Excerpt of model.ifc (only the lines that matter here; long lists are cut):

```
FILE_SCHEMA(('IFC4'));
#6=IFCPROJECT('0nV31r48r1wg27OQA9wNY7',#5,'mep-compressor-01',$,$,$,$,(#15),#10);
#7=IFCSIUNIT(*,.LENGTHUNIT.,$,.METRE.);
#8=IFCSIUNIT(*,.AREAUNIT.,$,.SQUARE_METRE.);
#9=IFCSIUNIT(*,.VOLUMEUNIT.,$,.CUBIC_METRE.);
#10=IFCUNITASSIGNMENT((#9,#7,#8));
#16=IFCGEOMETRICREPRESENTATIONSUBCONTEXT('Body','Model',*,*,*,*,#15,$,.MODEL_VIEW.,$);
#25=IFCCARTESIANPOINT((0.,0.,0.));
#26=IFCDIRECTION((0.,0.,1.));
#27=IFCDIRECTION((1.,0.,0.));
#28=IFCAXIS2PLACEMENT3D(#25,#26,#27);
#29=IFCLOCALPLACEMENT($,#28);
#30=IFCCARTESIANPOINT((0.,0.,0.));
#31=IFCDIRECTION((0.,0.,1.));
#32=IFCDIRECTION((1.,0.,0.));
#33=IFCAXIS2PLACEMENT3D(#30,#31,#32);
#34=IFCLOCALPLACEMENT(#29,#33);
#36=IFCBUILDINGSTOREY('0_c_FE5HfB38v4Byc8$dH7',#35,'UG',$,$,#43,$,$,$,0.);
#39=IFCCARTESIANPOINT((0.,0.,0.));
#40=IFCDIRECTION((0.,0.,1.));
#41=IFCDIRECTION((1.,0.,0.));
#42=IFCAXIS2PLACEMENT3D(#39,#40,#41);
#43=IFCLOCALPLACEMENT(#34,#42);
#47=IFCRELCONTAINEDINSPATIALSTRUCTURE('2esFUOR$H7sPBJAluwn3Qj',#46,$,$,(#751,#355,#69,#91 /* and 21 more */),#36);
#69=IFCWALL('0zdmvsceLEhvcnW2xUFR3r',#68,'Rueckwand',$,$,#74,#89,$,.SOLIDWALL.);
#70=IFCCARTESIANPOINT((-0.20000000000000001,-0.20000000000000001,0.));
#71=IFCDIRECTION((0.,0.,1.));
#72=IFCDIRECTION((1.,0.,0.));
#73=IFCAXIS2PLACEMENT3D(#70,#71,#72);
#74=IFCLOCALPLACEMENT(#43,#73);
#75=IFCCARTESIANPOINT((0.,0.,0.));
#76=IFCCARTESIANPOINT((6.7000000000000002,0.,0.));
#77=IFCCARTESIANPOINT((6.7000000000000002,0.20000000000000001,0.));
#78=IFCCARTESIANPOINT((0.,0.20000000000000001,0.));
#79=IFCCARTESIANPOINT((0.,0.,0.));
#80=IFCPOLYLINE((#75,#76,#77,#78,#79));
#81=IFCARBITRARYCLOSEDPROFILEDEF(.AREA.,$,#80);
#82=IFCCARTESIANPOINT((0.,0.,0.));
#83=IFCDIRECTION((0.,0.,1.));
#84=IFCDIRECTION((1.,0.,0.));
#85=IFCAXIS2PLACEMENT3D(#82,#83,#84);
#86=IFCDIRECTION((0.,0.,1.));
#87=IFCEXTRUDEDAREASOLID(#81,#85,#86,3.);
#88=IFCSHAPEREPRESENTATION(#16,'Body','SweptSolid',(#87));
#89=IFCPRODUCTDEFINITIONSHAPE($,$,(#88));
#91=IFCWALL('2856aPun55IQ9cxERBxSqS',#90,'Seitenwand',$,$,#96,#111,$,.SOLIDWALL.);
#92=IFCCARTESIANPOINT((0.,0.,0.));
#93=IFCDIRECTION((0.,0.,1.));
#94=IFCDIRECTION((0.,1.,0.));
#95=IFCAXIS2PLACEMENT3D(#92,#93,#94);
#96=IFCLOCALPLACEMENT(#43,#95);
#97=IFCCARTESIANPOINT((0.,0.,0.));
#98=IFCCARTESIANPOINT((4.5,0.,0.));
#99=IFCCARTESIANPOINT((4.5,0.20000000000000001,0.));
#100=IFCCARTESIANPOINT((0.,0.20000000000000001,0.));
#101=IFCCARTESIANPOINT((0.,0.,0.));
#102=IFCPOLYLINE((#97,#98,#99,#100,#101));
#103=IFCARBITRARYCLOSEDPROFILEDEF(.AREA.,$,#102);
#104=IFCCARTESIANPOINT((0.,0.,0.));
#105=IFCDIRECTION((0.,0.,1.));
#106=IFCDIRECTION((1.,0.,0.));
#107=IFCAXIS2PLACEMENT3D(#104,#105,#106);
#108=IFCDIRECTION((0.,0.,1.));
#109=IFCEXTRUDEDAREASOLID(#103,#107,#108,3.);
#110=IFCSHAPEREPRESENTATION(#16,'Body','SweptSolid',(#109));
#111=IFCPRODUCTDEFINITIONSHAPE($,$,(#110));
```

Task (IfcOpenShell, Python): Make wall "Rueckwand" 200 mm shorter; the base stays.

```python
import ifcopenshell
import ifcopenshell.geom
import ifcopenshell.util.representation
import ifcopenshell.util.shape

model = ifcopenshell.open("model.ifc")
settings = ifcopenshell.geom.settings()


def volume(element):
    """Net volume in cubic metres, openings subtracted."""
    shape = ifcopenshell.geom.create_shape(settings, element)
    return ifcopenshell.util.shape.get_volume(shape.geometry)


wall = model.by_guid("0zdmvsceLEhvcnW2xUFR3r")
before = volume(wall)

body = ifcopenshell.util.representation.get_representation(wall, "Model", "Body")
solid = body.Items[0]
old_height = solid.Depth
solid.Depth -= 0.2
after = volume(wall)

print(f"height {old_height:g} -> {solid.Depth:g}, volume {before:.3f} -> {after:.3f} m3")

model.write("model_v2.ifc")
```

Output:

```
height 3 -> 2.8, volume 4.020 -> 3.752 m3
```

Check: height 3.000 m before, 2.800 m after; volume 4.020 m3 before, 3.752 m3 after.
